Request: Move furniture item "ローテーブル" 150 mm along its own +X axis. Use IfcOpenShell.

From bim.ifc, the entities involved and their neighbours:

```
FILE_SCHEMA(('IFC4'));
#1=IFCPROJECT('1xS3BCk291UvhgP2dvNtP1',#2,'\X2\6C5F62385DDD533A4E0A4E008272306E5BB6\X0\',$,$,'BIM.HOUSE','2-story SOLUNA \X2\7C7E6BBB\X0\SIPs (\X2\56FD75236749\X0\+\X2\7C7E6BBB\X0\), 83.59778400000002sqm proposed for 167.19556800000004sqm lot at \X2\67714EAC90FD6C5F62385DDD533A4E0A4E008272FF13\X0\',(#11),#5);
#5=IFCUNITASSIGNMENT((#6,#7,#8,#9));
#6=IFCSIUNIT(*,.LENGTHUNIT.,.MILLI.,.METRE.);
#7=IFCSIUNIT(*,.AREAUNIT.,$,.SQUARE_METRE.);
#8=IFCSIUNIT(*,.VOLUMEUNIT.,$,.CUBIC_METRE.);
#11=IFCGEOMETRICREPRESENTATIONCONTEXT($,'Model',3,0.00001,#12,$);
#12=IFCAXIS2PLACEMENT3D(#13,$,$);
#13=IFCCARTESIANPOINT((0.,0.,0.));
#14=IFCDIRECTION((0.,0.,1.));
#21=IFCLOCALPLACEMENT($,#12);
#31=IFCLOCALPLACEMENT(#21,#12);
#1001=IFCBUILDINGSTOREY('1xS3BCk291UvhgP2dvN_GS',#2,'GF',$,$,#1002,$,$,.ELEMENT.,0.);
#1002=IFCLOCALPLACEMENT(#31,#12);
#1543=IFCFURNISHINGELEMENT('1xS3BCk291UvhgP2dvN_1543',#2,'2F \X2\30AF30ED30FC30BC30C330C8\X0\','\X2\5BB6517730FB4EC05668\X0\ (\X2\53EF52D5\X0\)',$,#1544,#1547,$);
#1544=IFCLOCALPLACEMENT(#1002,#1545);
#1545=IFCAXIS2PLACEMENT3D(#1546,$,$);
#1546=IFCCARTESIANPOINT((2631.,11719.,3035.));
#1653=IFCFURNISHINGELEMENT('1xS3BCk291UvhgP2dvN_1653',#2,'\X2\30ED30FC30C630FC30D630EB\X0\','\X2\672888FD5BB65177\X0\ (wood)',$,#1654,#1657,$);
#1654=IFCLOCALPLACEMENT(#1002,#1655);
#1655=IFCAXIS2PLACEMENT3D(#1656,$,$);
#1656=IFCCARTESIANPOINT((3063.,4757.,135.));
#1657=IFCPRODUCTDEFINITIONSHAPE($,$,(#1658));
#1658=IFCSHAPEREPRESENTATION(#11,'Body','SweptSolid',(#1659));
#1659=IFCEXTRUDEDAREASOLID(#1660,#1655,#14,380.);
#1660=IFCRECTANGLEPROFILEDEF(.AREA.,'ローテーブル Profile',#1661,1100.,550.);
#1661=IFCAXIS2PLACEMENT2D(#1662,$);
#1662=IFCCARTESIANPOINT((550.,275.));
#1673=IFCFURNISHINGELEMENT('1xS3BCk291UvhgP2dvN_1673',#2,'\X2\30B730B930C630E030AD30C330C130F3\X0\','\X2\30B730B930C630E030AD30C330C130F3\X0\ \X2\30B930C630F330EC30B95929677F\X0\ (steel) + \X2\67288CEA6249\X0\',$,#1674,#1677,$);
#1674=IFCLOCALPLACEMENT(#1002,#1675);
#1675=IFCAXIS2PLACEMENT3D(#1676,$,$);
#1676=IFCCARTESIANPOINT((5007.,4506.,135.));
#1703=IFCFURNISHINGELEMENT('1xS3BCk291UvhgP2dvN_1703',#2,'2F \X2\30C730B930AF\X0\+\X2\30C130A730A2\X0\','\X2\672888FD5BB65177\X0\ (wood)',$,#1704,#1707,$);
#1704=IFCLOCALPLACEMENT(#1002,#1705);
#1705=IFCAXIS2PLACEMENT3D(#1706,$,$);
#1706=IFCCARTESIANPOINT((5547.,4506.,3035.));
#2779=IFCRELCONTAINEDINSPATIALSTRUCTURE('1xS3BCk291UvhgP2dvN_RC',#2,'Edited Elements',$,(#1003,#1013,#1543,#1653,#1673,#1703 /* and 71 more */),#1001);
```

```python
import ifcopenshell
import ifcopenshell.api.geometry
import ifcopenshell.util.placement
import ifcopenshell.util.unit

model = ifcopenshell.open("bim.ifc")
unit_scale = ifcopenshell.util.unit.calculate_unit_scale(model)

item = model.by_guid("1xS3BCk291UvhgP2dvN_1653")
matrix = ifcopenshell.util.placement.get_local_placement(item.ObjectPlacement)
matrix[:3, 3] += matrix[:3, 0] * 0.15 / unit_scale
ifcopenshell.api.geometry.edit_object_placement(model, product=item, matrix=matrix, is_si=False)

print(ifcopenshell.util.placement.get_local_placement(item.ObjectPlacement).round(3) + 0.0)

model.write("bim_rev.ifc")
```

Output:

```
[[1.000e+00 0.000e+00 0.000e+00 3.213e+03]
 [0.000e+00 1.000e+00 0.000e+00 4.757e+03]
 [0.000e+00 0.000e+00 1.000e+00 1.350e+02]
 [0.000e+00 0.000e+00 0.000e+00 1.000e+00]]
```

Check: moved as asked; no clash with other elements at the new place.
